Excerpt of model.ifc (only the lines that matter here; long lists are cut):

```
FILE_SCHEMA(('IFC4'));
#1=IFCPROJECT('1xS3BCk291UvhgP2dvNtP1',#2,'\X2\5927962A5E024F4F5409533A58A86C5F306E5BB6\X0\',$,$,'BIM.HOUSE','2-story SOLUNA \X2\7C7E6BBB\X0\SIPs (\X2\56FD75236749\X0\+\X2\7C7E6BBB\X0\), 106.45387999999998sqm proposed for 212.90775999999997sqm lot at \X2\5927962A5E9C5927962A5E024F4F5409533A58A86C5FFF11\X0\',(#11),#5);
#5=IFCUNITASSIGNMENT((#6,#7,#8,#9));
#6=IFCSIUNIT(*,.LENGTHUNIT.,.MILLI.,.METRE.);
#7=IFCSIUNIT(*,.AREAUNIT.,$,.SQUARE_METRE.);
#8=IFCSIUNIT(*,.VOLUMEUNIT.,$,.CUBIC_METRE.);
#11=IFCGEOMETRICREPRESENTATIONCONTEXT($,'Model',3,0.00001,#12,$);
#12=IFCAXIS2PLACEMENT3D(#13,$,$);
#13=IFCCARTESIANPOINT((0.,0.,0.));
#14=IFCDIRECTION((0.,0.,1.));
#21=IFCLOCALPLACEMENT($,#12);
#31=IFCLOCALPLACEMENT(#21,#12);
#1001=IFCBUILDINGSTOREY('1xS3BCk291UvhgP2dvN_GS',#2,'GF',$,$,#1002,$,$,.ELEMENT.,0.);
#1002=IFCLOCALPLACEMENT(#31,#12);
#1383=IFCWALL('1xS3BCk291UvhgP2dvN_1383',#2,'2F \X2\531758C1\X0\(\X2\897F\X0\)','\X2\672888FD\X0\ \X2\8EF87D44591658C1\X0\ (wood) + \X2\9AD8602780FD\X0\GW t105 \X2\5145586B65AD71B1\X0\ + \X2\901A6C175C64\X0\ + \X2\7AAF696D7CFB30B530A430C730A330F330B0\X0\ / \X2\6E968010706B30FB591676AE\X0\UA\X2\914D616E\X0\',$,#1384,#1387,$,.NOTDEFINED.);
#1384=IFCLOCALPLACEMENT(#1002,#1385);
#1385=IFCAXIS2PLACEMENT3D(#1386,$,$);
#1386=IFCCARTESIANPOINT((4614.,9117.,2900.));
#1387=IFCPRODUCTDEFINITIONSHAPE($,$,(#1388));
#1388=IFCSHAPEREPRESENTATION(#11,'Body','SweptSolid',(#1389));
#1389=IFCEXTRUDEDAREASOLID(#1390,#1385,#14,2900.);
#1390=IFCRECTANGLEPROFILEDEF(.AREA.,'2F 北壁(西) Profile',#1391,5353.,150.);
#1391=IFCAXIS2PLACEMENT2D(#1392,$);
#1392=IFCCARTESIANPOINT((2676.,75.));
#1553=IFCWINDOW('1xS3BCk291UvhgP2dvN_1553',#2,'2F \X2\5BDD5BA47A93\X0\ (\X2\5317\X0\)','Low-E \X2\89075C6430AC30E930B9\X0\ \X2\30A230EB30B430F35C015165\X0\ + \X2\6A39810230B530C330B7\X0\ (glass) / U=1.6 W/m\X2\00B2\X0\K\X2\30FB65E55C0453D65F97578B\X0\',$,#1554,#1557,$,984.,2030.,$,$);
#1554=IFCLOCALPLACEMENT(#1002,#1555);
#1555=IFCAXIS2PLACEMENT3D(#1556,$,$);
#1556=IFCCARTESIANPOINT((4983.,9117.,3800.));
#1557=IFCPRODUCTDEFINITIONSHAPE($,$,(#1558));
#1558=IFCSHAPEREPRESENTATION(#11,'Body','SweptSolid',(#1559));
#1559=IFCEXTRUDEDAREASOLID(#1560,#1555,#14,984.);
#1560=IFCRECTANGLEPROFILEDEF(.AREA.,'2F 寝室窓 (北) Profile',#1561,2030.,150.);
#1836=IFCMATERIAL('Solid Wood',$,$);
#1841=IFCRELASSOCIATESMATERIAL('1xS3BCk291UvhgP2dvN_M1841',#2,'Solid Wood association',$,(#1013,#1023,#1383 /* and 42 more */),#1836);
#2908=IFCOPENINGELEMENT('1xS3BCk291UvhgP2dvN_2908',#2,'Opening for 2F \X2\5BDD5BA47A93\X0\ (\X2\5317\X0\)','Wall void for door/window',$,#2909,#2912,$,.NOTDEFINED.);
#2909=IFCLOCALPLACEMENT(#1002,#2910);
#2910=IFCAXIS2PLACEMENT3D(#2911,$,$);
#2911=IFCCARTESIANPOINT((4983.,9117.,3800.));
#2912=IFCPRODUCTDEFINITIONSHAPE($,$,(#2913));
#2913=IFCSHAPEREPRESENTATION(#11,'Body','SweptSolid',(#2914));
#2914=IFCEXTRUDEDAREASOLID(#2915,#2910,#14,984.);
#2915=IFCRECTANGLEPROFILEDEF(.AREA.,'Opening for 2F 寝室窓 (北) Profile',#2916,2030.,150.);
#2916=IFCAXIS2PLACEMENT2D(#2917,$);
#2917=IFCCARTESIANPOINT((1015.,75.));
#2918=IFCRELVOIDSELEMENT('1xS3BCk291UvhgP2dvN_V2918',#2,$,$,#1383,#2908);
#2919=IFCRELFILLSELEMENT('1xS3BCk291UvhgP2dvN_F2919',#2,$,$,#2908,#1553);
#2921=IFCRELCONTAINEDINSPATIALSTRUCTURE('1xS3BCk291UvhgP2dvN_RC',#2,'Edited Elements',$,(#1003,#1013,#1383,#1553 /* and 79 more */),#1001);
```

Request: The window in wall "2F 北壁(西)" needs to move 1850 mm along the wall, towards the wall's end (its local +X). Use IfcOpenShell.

```python
import ifcopenshell
import ifcopenshell.api.geometry
import ifcopenshell.util.placement

model = ifcopenshell.open("model.ifc")

window = model.by_id(1553)
opening = window.FillsVoids[0].RelatingOpeningElement
wall = opening.VoidsElements[0].RelatingBuildingElement

wall_matrix = ifcopenshell.util.placement.get_local_placement(wall.ObjectPlacement)
shift = wall_matrix[:3, 0] * 1850.0
before = ifcopenshell.util.placement.get_local_placement(window.ObjectPlacement)[:3, 3].copy()

# The window is not placed relative to its opening, so move both.
for product in (opening, window):
    matrix = ifcopenshell.util.placement.get_local_placement(product.ObjectPlacement)
    matrix[:3, 3] += shift
    ifcopenshell.api.geometry.edit_object_placement(model, product=product, matrix=matrix, is_si=False)

after = ifcopenshell.util.placement.get_local_placement(window.ObjectPlacement)[:3, 3]
print("window moved by", (after - before).round(3) + 0.0)

model.write("model_updated.ifc")
```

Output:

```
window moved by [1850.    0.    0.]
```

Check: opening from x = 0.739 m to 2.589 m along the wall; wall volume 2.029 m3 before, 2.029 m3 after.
